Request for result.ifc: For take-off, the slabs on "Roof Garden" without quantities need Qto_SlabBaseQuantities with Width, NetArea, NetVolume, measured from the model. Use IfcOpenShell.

First a look at what the model holds.

```python
import ifcopenshell
import ifcopenshell.util.element
import ifcopenshell.util.unit

model = ifcopenshell.open("result.ifc")
print(model.schema)
for unit_type in ("LENGTHUNIT", "AREAUNIT", "VOLUMEUNIT"):
    print(unit_type, ifcopenshell.util.unit.calculate_unit_scale(model, unit_type))
storey = next(s for s in model.by_type("IfcBuildingStorey") if s.Name == "Roof Garden")
slabs = [e for e in ifcopenshell.util.element.get_decomposition(storey) if e.is_a("IfcSlab")]
for e in sorted(slabs, key=lambda e: e.id()):
    print(e.id(), e.is_a(), e.Name, list(ifcopenshell.util.element.get_psets(e, qtos_only=True)), sep=" | ")
```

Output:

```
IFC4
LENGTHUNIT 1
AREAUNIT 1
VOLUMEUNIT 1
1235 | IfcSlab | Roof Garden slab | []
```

```python
import ifcopenshell
import ifcopenshell.api.pset
import ifcopenshell.geom
import ifcopenshell.util.element
import ifcopenshell.util.shape
import ifcopenshell.util.unit

model = ifcopenshell.open("result.ifc")
unit_scale = ifcopenshell.util.unit.calculate_unit_scale(model)
area_scale = ifcopenshell.util.unit.calculate_unit_scale(model, "AREAUNIT")
volume_scale = ifcopenshell.util.unit.calculate_unit_scale(model, "VOLUMEUNIT")
settings = ifcopenshell.geom.settings()

storey = next(s for s in model.by_type("IfcBuildingStorey") if s.Name == "Roof Garden")
slabs = [e for e in ifcopenshell.util.element.get_decomposition(storey) if e.is_a("IfcSlab")]

for e in sorted(slabs, key=lambda e: e.id()):
    if ifcopenshell.util.element.get_psets(e, qtos_only=True, should_inherit=False):
        continue
    # Geometry comes back in metres, in the element's own axes.
    shape = ifcopenshell.geom.create_shape(settings, e)
    values = {
        "Width": ifcopenshell.util.shape.get_z(shape.geometry) / unit_scale,
        "NetArea": ifcopenshell.util.shape.get_footprint_area(shape.geometry) / area_scale,
        "NetVolume": ifcopenshell.util.shape.get_volume(shape.geometry) / volume_scale,
    }
    qto = ifcopenshell.api.pset.add_qto(model, product=e, name="Qto_SlabBaseQuantities")
    ifcopenshell.api.pset.edit_qto(model, qto=qto, properties=values)
    print(e.id(), {k: round(v, 3) for k, v in values.items()})

model.write("result_rev.ifc")
```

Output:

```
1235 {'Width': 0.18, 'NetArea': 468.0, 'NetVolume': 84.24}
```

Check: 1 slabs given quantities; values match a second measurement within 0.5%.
